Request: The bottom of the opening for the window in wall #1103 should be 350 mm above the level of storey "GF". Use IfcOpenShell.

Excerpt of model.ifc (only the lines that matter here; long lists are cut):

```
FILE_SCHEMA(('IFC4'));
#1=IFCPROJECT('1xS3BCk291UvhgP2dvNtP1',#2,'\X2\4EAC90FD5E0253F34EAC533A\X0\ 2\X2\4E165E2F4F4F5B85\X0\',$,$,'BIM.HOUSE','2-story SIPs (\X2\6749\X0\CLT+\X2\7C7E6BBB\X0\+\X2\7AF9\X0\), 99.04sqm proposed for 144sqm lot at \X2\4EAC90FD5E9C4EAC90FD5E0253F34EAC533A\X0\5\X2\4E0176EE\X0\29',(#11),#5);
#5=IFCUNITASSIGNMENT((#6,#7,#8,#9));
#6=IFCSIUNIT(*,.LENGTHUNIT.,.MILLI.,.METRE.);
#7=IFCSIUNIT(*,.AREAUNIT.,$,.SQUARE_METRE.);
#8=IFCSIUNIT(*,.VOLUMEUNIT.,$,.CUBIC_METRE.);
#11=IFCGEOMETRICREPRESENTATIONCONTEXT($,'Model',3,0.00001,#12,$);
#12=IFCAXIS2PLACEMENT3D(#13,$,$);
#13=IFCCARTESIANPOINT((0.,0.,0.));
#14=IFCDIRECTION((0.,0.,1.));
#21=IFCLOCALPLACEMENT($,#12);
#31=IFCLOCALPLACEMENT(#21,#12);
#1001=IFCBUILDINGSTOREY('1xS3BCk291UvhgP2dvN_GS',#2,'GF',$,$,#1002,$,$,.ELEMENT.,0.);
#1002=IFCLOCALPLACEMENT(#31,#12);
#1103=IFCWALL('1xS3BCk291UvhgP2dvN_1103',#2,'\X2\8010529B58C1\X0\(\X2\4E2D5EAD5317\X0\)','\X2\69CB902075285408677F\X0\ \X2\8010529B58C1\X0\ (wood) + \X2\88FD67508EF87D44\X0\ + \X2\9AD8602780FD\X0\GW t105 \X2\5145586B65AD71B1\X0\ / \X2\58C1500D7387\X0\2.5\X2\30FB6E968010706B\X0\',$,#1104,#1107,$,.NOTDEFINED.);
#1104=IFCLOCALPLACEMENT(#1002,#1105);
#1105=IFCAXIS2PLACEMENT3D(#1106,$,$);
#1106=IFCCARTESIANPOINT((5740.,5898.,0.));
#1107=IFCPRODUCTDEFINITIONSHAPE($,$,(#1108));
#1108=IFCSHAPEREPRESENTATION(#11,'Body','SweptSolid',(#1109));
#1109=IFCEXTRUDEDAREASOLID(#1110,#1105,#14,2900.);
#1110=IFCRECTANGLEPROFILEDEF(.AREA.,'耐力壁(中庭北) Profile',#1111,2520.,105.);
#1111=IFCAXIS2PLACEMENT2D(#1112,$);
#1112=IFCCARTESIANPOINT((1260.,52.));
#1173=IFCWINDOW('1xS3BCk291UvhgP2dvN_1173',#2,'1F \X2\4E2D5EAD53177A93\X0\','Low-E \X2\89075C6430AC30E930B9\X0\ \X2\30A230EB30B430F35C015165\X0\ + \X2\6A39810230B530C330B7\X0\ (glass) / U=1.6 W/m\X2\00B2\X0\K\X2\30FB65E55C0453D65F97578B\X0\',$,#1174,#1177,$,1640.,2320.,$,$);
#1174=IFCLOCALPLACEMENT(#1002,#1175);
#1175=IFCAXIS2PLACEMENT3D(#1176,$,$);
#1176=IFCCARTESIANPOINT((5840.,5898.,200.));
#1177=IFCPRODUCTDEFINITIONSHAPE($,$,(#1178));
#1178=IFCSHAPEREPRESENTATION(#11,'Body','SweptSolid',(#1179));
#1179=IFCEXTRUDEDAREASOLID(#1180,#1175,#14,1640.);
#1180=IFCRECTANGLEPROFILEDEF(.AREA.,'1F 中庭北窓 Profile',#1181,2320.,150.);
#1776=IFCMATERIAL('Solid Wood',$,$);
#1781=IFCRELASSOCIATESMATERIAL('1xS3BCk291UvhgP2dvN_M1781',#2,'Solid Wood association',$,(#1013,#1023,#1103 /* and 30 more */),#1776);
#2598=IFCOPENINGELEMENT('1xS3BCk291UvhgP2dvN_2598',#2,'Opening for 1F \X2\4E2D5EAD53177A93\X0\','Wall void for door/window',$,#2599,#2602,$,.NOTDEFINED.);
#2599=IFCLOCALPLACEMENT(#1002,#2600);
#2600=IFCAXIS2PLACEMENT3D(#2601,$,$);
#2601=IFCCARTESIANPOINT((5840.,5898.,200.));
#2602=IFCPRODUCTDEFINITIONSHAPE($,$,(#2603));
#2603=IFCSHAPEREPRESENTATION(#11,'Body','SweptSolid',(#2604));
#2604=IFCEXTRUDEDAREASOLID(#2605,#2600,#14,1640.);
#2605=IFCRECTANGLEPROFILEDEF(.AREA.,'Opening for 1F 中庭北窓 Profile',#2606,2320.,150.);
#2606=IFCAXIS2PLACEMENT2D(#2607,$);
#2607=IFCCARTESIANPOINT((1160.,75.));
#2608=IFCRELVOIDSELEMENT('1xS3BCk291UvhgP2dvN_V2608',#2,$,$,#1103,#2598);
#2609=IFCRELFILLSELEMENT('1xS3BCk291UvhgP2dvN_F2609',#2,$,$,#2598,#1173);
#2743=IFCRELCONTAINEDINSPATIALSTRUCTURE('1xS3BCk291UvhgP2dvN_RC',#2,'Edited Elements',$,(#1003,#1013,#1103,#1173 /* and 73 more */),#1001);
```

```python
import numpy as np
import ifcopenshell
import ifcopenshell.api.geometry
import ifcopenshell.geom
import ifcopenshell.util.element
import ifcopenshell.util.placement
import ifcopenshell.util.shape
import ifcopenshell.util.unit

model = ifcopenshell.open("model.ifc")
unit_scale = ifcopenshell.util.unit.calculate_unit_scale(model)

window = model.by_guid("1xS3BCk291UvhgP2dvN_1173")
opening = window.FillsVoids[0].RelatingOpeningElement
storey = ifcopenshell.util.element.get_container(window, ifc_class="IfcBuildingStorey")
level = ifcopenshell.util.placement.get_local_placement(storey.ObjectPlacement)[2, 3]

# The opening's origin need not be at the sill, so measure its lowest point.
shape = ifcopenshell.geom.create_shape(ifcopenshell.geom.settings(), opening)
bottom = ifcopenshell.util.shape.get_shape_bottom_elevation(shape, shape.geometry) / unit_scale
dz = level + 350.0 - bottom

shift = np.array([0.0, 0.0, dz])
# The window is not placed relative to its opening, so move both.
for product in (opening, window):
    matrix = ifcopenshell.util.placement.get_local_placement(product.ObjectPlacement)
    matrix[:3, 3] += shift
    ifcopenshell.api.geometry.edit_object_placement(model, product=product, matrix=matrix, is_si=False)

print(f"moved by {dz * unit_scale:+.3f} m")

model.write("model_rev.ifc")
```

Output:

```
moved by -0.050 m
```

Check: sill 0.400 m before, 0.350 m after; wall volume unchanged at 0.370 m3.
